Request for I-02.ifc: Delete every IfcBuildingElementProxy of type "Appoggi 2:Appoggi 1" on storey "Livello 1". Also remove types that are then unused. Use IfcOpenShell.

First a look at what the model holds.

```python
import ifcopenshell
import ifcopenshell.util.element

model = ifcopenshell.open("I-02.ifc")
print(model.schema)
storey = next(s for s in model.by_type("IfcBuildingStorey") if s.Name == "Livello 1")
proxies = [e for e in ifcopenshell.util.element.get_decomposition(storey) if e.is_a("IfcBuildingElementProxy")]
seen = {}
for e in proxies:
    element_type = ifcopenshell.util.element.get_type(e)
    name = element_type.Name if element_type not in (None, e) else None
    seen[name] = seen.get(name, 0) + 1
for name, count in sorted(seen.items(), key=str):
    print(count, "x", name)
```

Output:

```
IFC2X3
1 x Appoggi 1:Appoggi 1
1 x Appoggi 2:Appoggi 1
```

```python
import ifcopenshell
import ifcopenshell.api.root
import ifcopenshell.util.element

model = ifcopenshell.open("I-02.ifc")

storey = next(s for s in model.by_type("IfcBuildingStorey") if s.Name == "Livello 1")
proxies = [e for e in ifcopenshell.util.element.get_decomposition(storey) if e.is_a("IfcBuildingElementProxy")]
targets = [e for e in proxies if (t := ifcopenshell.util.element.get_type(e)) not in (None, e) and t.Name == "Appoggi 2:Appoggi 1"]
types = {ifcopenshell.util.element.get_type(e) for e in targets} - {None, *targets}

for e in targets:
    ifcopenshell.api.root.remove_product(model, product=e)
print(len(targets), "removed")

unused = [t for t in types if not ifcopenshell.util.element.get_types(t)]
for t in unused:
    ifcopenshell.api.root.remove_product(model, product=t)
print(len(unused), "unused types removed")

model.write("I-02-out.ifc")
```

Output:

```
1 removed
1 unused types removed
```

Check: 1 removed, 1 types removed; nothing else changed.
